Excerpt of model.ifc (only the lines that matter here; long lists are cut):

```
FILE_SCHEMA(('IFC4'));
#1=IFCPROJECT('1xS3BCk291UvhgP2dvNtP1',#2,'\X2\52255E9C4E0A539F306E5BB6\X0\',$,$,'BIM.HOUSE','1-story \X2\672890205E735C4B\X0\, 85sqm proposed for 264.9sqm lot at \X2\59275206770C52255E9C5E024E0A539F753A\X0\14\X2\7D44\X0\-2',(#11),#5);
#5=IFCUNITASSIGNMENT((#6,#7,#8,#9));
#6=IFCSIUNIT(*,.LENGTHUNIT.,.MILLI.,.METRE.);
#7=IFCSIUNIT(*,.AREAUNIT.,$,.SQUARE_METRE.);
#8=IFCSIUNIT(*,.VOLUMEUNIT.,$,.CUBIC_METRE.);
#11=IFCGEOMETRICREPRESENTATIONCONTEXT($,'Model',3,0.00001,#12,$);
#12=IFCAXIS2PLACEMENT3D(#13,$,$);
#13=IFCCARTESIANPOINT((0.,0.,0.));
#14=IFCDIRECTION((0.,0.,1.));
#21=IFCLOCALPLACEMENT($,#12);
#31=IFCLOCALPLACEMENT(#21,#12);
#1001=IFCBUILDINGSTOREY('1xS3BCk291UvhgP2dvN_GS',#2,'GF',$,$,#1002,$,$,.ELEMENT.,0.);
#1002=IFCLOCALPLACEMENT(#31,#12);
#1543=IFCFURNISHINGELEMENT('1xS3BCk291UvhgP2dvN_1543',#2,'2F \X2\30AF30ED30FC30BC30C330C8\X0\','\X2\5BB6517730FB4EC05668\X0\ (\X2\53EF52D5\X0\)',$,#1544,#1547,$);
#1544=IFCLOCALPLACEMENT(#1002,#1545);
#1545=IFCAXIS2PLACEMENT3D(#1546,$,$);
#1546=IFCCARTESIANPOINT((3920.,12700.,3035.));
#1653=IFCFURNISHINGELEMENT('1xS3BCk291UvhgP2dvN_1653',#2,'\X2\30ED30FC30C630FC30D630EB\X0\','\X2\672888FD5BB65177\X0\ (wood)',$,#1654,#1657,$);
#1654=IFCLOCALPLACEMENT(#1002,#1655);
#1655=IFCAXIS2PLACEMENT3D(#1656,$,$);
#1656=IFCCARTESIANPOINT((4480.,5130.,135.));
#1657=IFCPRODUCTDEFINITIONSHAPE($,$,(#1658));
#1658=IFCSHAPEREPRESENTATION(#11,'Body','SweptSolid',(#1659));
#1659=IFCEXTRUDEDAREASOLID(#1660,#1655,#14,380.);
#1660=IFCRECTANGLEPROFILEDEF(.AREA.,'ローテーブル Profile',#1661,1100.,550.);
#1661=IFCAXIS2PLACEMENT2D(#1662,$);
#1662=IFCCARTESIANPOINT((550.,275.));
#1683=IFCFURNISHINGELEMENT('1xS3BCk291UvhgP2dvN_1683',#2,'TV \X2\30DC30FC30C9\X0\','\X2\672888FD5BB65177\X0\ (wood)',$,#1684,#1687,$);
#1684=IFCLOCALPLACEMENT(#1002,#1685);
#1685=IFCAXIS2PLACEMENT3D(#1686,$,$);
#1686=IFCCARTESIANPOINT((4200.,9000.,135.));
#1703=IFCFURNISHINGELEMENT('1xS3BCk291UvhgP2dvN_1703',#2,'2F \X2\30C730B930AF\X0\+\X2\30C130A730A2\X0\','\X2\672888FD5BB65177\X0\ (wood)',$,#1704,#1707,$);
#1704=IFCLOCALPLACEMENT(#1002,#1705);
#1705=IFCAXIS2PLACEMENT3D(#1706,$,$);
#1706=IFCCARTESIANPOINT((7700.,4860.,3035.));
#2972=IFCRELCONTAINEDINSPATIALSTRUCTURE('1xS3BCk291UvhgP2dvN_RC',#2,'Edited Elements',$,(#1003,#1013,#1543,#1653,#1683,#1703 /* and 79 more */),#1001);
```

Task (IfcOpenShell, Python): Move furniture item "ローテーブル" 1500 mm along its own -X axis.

```python
import ifcopenshell
import ifcopenshell.api.geometry
import ifcopenshell.util.placement
import ifcopenshell.util.unit

model = ifcopenshell.open("model.ifc")
unit_scale = ifcopenshell.util.unit.calculate_unit_scale(model)

item = model.by_guid("1xS3BCk291UvhgP2dvN_1653")
matrix = ifcopenshell.util.placement.get_local_placement(item.ObjectPlacement)
matrix[:3, 3] -= matrix[:3, 0] * 1.5 / unit_scale
ifcopenshell.api.geometry.edit_object_placement(model, product=item, matrix=matrix, is_si=False)

print(ifcopenshell.util.placement.get_local_placement(item.ObjectPlacement).round(3) + 0.0)

model.write("model_rev.ifc")
```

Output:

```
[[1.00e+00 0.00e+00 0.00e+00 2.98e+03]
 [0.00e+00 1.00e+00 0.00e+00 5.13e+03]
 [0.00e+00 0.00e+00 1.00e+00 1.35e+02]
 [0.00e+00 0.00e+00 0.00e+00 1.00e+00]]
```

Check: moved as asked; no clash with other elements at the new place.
